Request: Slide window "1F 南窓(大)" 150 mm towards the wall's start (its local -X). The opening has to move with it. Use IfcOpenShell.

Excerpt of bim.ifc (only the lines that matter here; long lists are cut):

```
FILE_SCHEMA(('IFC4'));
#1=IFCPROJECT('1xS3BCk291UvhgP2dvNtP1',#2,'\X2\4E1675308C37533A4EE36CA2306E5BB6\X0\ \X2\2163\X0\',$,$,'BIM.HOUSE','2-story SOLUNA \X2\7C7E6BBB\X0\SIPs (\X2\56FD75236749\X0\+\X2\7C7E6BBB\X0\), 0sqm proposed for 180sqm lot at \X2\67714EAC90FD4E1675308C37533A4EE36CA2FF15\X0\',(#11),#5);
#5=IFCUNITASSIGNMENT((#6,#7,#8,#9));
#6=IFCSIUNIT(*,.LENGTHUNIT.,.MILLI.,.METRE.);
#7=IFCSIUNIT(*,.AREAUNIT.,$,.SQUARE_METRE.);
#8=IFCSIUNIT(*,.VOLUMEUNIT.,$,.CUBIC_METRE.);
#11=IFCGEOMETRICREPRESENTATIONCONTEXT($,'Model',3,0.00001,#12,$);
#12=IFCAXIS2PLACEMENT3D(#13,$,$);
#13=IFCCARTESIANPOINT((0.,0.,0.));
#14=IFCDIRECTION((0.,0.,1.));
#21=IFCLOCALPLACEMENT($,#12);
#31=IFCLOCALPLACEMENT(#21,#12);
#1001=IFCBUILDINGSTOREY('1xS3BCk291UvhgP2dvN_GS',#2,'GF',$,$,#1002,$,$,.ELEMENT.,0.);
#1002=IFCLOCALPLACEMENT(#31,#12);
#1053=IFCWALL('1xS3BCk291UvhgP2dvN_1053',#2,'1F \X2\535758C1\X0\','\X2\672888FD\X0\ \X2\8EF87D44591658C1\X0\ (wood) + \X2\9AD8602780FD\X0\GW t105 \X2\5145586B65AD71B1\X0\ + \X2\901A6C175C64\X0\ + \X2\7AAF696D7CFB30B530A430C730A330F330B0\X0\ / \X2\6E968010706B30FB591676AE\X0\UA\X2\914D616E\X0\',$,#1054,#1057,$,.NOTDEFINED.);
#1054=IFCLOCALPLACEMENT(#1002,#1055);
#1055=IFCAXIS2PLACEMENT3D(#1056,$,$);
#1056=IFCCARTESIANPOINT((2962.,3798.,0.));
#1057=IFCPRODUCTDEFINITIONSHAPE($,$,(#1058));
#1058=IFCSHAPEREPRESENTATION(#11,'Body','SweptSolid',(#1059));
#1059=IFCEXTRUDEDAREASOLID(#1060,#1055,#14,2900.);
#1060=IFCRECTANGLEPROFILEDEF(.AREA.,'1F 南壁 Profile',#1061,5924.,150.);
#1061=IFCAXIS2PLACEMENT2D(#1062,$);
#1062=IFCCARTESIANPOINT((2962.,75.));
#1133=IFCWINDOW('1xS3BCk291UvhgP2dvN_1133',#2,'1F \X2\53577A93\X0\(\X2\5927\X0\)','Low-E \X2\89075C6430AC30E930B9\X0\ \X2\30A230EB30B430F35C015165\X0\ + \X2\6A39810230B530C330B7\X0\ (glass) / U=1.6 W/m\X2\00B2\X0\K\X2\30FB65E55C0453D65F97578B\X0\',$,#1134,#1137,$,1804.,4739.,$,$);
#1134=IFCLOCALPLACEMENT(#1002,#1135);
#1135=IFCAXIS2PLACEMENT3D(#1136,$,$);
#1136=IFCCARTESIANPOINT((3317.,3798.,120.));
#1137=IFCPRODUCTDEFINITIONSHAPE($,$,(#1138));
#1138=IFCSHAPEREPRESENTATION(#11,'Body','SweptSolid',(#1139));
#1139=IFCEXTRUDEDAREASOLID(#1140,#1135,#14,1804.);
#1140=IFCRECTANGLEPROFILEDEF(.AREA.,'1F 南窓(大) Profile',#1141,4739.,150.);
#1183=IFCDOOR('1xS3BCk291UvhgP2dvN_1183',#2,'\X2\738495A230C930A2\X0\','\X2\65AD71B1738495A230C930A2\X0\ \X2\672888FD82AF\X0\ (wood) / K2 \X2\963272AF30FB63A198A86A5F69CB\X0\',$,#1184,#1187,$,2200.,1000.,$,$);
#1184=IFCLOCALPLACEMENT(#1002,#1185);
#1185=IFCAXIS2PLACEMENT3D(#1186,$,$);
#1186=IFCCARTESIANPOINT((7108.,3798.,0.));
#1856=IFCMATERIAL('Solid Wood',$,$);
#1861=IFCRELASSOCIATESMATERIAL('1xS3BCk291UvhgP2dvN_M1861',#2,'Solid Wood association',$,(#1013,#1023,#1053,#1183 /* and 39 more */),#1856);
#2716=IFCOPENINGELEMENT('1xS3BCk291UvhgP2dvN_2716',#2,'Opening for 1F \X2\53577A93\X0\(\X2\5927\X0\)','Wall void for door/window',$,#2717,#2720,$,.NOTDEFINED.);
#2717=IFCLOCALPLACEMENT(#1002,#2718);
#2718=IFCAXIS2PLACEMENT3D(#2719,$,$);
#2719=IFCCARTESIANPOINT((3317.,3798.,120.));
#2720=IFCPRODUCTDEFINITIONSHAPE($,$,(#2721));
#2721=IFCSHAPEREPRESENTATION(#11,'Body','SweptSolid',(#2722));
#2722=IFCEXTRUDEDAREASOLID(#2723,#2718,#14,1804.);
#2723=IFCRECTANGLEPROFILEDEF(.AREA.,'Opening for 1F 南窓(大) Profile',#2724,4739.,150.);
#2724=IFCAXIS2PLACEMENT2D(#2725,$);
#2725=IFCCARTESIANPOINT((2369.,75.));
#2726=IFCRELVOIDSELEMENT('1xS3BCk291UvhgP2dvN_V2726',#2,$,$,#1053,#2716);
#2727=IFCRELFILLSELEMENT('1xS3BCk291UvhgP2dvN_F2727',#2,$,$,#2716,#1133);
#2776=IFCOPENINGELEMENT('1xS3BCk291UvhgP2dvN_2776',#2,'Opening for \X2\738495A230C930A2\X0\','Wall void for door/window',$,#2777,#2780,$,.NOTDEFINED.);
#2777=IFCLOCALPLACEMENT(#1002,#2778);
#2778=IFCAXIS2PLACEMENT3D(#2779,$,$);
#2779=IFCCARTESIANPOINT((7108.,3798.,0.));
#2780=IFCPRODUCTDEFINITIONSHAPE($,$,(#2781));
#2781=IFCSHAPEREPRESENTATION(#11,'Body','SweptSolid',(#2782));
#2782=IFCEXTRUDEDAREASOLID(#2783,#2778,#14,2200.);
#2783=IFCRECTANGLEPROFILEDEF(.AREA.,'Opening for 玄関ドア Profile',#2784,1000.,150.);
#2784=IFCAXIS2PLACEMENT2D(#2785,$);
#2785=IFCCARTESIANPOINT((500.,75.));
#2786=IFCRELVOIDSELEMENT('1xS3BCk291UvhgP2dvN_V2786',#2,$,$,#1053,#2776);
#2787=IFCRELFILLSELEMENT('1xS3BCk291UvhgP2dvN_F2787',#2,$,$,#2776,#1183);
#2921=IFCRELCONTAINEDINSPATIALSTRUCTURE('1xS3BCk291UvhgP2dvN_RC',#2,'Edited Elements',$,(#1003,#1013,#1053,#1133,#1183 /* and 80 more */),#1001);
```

```python
import ifcopenshell
import ifcopenshell.api.geometry
import ifcopenshell.util.placement
import ifcopenshell.util.unit

model = ifcopenshell.open("bim.ifc")
unit_scale = ifcopenshell.util.unit.calculate_unit_scale(model)

window = model.by_guid("1xS3BCk291UvhgP2dvN_1133")
opening = window.FillsVoids[0].RelatingOpeningElement
wall = opening.VoidsElements[0].RelatingBuildingElement

wall_matrix = ifcopenshell.util.placement.get_local_placement(wall.ObjectPlacement)
shift = wall_matrix[:3, 0] * -0.15 / unit_scale
before = ifcopenshell.util.placement.get_local_placement(window.ObjectPlacement)[:3, 3].copy()

# The window is not placed relative to its opening, so move both.
for product in (opening, window):
    matrix = ifcopenshell.util.placement.get_local_placement(product.ObjectPlacement)
    matrix[:3, 3] += shift
    ifcopenshell.api.geometry.edit_object_placement(model, product=product, matrix=matrix, is_si=False)

after = ifcopenshell.util.placement.get_local_placement(window.ObjectPlacement)[:3, 3]
print("window moved by", (after - before).round(3) + 0.0)

model.write("bim_v2.ifc")
```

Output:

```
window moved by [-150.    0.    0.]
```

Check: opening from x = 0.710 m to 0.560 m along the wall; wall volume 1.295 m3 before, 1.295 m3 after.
